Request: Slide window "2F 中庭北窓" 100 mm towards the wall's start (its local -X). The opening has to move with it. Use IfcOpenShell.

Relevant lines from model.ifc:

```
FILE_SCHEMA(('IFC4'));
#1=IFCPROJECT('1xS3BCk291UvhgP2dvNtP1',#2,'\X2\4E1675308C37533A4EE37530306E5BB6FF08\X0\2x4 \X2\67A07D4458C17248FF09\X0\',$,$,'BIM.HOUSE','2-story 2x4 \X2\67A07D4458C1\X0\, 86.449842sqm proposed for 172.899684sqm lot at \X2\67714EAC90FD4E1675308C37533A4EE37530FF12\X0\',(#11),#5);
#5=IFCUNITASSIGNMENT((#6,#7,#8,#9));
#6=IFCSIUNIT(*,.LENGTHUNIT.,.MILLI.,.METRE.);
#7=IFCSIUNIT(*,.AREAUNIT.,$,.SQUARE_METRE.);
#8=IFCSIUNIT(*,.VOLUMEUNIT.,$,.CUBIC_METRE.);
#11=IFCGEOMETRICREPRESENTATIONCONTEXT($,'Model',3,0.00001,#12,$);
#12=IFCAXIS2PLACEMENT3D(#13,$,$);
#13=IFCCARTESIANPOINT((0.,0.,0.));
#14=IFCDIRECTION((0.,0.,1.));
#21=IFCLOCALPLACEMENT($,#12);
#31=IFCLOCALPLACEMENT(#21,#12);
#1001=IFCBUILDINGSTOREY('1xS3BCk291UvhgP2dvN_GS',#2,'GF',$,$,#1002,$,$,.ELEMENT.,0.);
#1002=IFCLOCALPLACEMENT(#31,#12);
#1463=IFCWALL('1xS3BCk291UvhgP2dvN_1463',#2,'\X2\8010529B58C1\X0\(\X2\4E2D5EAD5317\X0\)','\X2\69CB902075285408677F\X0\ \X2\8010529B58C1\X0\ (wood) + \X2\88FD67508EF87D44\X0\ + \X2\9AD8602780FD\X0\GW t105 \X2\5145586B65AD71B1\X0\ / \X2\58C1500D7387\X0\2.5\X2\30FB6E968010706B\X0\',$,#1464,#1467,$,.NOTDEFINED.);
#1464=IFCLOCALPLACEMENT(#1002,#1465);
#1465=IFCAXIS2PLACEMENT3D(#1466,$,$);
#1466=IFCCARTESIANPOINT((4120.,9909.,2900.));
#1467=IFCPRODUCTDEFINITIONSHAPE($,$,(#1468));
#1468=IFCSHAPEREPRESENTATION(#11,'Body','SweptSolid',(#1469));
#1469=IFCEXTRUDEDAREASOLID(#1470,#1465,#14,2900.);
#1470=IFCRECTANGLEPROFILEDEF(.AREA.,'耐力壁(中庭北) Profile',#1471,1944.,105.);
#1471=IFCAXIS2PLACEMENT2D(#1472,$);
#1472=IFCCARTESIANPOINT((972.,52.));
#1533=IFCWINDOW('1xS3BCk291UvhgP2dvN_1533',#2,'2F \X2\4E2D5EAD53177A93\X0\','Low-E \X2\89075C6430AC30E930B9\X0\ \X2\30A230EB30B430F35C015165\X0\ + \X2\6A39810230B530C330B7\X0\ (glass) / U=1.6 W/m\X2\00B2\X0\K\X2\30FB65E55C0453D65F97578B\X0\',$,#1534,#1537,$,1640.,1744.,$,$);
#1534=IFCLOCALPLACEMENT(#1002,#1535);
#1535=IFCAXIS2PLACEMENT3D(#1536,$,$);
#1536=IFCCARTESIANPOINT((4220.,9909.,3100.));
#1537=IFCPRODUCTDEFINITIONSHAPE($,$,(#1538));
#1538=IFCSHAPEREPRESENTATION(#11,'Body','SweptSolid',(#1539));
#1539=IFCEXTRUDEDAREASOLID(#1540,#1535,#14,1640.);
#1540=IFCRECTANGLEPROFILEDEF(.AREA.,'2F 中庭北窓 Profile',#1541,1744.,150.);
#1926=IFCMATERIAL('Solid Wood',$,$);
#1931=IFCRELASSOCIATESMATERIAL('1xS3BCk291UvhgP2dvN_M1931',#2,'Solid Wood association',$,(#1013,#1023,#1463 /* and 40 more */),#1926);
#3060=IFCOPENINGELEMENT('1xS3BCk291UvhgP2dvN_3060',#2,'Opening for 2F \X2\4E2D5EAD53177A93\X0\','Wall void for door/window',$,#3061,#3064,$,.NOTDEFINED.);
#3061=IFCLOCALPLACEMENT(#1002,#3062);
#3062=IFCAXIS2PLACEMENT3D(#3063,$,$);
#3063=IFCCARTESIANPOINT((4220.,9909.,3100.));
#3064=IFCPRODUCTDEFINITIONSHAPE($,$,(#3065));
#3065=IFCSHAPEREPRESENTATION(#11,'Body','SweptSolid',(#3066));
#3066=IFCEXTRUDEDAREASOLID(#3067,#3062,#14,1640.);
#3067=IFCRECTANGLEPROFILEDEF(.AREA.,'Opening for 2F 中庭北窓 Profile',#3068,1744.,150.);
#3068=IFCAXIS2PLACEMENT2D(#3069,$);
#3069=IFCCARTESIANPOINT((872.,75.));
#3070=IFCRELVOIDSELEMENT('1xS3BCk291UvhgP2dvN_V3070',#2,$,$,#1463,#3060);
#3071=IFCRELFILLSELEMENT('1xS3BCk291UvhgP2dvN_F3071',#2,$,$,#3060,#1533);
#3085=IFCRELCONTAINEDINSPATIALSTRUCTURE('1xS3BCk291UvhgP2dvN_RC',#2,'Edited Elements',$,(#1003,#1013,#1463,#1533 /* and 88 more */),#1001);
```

```python
import ifcopenshell
import ifcopenshell.api.geometry
import ifcopenshell.util.placement
import ifcopenshell.util.unit

model = ifcopenshell.open("model.ifc")
unit_scale = ifcopenshell.util.unit.calculate_unit_scale(model)

window = model.by_id(1533)
opening = window.FillsVoids[0].RelatingOpeningElement
wall = opening.VoidsElements[0].RelatingBuildingElement

wall_matrix = ifcopenshell.util.placement.get_local_placement(wall.ObjectPlacement)
shift = wall_matrix[:3, 0] * -0.1 / unit_scale
before = ifcopenshell.util.placement.get_local_placement(window.ObjectPlacement)[:3, 3].copy()

# The window is not placed relative to its opening, so move both.
for product in (opening, window):
    matrix = ifcopenshell.util.placement.get_local_placement(product.ObjectPlacement)
    matrix[:3, 3] += shift
    ifcopenshell.api.geometry.edit_object_placement(model, product=product, matrix=matrix, is_si=False)

after = ifcopenshell.util.placement.get_local_placement(window.ObjectPlacement)[:3, 3]
print("window moved by", (after - before).round(3) + 0.0)

model.write("model_updated.ifc")
```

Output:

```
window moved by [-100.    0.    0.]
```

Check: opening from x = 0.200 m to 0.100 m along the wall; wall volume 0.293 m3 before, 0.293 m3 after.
